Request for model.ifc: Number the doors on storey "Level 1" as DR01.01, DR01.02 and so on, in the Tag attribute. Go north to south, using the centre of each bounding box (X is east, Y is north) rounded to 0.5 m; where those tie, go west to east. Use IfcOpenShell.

First a look at what the model holds.

```python
import ifcopenshell
import ifcopenshell.util.element
import ifcopenshell.util.placement

model = ifcopenshell.open("model.ifc")
print(model.schema)
storey = next(s for s in model.by_type("IfcBuildingStorey") if s.Name == "Level 1")
doors = [e for e in ifcopenshell.util.element.get_decomposition(storey) if e.is_a("IfcDoor")]
for e in sorted(doors, key=lambda e: e.id()):
    origin = ifcopenshell.util.placement.get_local_placement(e.ObjectPlacement)[:3, 3]
    print(e.id(), e.Tag, e.Name, origin.round(2) + 0.0, sep=" | ")
```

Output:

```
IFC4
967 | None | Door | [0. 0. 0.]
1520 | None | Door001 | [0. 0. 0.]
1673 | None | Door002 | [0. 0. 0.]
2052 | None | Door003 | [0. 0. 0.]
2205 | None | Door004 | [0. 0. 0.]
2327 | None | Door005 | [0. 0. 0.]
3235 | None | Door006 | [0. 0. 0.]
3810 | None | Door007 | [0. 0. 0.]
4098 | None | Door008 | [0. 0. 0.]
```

```python
import ifcopenshell
import ifcopenshell.geom
import ifcopenshell.util.element
import ifcopenshell.util.shape

model = ifcopenshell.open("model.ifc")
settings = ifcopenshell.geom.settings()
settings.set("use-world-coords", True)


def centre(element):
    shape = ifcopenshell.geom.create_shape(settings, element)
    return ifcopenshell.util.shape.get_bbox_centroid(shape.geometry)


storey = next(s for s in model.by_type("IfcBuildingStorey") if s.Name == "Level 1")
doors = [e for e in ifcopenshell.util.element.get_decomposition(storey) if e.is_a("IfcDoor")]

# Insertion points can sit at a corner or the storey origin, so sort by the geometry (in metres).
centres = {e: centre(e) for e in doors}
doors.sort(key=lambda e: (-round(centres[e][1] / 0.5), centres[e][0]))

for i, e in enumerate(doors, start=1):
    number = f"DR01.{i:02d}"
    e.Tag = number
    print(e.id(), number)

model.write("model_v2.ifc")
```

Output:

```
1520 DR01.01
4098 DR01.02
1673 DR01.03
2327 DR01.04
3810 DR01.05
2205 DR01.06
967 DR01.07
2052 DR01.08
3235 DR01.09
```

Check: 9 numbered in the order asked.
